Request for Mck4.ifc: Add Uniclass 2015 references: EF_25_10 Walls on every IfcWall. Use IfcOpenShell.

First a look at what the model holds.

```python
import ifcopenshell

model = ifcopenshell.open("Mck4.ifc")
print(model.schema)
print("classifications:", [c.Name for c in model.by_type("IfcClassification")])
for ifc_class in ("IfcDoor", "IfcRoof", "IfcStair", "IfcWall", "IfcWindow"):
    print(ifc_class, len(model.by_type(ifc_class)))
```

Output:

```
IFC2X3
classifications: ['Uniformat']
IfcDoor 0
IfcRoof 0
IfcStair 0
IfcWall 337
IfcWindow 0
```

```python
import ifcopenshell
import ifcopenshell.api.classification

model = ifcopenshell.open("Mck4.ifc")

# IFC2X3 requires Source and Edition and has no link from the project to the system.
system = model.create_entity("IfcClassification", Source="NBS", Edition="2015", Name="Uniclass 2015")

codes = {
    "IfcWall": ("EF_25_10", "Walls"),
}
for ifc_class, (code, name) in codes.items():
    products = model.by_type(ifc_class)
    ifcopenshell.api.classification.add_reference(
        model, products=products, classification=system, identification=code, name=name
    )
    print(code, len(products))

model.write("Mck4_updated.ifc")
```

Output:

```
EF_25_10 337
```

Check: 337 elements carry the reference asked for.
